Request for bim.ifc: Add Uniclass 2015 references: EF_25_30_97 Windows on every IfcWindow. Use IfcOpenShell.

First a look at what the model holds.

```python
import ifcopenshell

model = ifcopenshell.open("bim.ifc")
print(model.schema)
print("classifications:", [c.Name for c in model.by_type("IfcClassification")])
for ifc_class in ("IfcDoor", "IfcRoof", "IfcStair", "IfcWall", "IfcWindow"):
    print(ifc_class, len(model.by_type(ifc_class)))
```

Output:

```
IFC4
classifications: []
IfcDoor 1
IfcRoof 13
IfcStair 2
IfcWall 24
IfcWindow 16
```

```python
import ifcopenshell
import ifcopenshell.api.classification

model = ifcopenshell.open("bim.ifc")

system = ifcopenshell.api.classification.add_classification(model, classification="Uniclass 2015")

codes = {
    "IfcWindow": ("EF_25_30_97", "Windows"),
}
for ifc_class, (code, name) in codes.items():
    products = model.by_type(ifc_class)
    ifcopenshell.api.classification.add_reference(
        model, products=products, classification=system, identification=code, name=name
    )
    print(code, len(products))

model.write("bim_rev.ifc")
```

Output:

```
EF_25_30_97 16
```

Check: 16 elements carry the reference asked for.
